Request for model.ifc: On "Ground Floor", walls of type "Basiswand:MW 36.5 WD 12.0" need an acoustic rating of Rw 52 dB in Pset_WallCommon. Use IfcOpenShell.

First a look at what the model holds.

```python
import ifcopenshell
import ifcopenshell.util.element

model = ifcopenshell.open("model.ifc")
print(model.schema)
storey = next(s for s in model.by_type("IfcBuildingStorey") if s.Name == "Ground Floor")
walls = [e for e in ifcopenshell.util.element.get_decomposition(storey) if e.is_a("IfcWall")]
seen = {}
for e in walls:
    element_type = ifcopenshell.util.element.get_type(e)
    key = (element_type.Name if element_type != e and element_type else None, ifcopenshell.util.element.get_pset(e, "Pset_WallCommon", "AcousticRating"))
    seen[key] = seen.get(key, 0) + 1
for (name, value), count in sorted(seen.items(), key=str):
    print(count, "x", name, "|", value)
```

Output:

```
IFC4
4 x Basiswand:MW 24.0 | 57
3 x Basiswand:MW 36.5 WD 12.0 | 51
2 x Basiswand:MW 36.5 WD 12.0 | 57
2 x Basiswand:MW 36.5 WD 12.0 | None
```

```python
import ifcopenshell
import ifcopenshell.api.pset
import ifcopenshell.util.element

model = ifcopenshell.open("model.ifc")

storey = next(s for s in model.by_type("IfcBuildingStorey") if s.Name == "Ground Floor")
walls = [e for e in ifcopenshell.util.element.get_decomposition(storey) if e.is_a("IfcWall")]

count = 0
for e in walls:
    element_type = ifcopenshell.util.element.get_type(e)
    if element_type in (None, e) or element_type.Name != "Basiswand:MW 36.5 WD 12.0":
        continue
    # add_pset returns the element's existing set when there is one.
    pset = ifcopenshell.api.pset.add_pset(model, product=e, name="Pset_WallCommon")
    ifcopenshell.api.pset.edit_pset(model, pset=pset, properties={"AcousticRating": "Rw 52 dB"})
    count += 1

print(count, "walls updated")

model.write("model_v2.ifc")
```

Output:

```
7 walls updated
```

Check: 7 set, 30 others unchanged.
